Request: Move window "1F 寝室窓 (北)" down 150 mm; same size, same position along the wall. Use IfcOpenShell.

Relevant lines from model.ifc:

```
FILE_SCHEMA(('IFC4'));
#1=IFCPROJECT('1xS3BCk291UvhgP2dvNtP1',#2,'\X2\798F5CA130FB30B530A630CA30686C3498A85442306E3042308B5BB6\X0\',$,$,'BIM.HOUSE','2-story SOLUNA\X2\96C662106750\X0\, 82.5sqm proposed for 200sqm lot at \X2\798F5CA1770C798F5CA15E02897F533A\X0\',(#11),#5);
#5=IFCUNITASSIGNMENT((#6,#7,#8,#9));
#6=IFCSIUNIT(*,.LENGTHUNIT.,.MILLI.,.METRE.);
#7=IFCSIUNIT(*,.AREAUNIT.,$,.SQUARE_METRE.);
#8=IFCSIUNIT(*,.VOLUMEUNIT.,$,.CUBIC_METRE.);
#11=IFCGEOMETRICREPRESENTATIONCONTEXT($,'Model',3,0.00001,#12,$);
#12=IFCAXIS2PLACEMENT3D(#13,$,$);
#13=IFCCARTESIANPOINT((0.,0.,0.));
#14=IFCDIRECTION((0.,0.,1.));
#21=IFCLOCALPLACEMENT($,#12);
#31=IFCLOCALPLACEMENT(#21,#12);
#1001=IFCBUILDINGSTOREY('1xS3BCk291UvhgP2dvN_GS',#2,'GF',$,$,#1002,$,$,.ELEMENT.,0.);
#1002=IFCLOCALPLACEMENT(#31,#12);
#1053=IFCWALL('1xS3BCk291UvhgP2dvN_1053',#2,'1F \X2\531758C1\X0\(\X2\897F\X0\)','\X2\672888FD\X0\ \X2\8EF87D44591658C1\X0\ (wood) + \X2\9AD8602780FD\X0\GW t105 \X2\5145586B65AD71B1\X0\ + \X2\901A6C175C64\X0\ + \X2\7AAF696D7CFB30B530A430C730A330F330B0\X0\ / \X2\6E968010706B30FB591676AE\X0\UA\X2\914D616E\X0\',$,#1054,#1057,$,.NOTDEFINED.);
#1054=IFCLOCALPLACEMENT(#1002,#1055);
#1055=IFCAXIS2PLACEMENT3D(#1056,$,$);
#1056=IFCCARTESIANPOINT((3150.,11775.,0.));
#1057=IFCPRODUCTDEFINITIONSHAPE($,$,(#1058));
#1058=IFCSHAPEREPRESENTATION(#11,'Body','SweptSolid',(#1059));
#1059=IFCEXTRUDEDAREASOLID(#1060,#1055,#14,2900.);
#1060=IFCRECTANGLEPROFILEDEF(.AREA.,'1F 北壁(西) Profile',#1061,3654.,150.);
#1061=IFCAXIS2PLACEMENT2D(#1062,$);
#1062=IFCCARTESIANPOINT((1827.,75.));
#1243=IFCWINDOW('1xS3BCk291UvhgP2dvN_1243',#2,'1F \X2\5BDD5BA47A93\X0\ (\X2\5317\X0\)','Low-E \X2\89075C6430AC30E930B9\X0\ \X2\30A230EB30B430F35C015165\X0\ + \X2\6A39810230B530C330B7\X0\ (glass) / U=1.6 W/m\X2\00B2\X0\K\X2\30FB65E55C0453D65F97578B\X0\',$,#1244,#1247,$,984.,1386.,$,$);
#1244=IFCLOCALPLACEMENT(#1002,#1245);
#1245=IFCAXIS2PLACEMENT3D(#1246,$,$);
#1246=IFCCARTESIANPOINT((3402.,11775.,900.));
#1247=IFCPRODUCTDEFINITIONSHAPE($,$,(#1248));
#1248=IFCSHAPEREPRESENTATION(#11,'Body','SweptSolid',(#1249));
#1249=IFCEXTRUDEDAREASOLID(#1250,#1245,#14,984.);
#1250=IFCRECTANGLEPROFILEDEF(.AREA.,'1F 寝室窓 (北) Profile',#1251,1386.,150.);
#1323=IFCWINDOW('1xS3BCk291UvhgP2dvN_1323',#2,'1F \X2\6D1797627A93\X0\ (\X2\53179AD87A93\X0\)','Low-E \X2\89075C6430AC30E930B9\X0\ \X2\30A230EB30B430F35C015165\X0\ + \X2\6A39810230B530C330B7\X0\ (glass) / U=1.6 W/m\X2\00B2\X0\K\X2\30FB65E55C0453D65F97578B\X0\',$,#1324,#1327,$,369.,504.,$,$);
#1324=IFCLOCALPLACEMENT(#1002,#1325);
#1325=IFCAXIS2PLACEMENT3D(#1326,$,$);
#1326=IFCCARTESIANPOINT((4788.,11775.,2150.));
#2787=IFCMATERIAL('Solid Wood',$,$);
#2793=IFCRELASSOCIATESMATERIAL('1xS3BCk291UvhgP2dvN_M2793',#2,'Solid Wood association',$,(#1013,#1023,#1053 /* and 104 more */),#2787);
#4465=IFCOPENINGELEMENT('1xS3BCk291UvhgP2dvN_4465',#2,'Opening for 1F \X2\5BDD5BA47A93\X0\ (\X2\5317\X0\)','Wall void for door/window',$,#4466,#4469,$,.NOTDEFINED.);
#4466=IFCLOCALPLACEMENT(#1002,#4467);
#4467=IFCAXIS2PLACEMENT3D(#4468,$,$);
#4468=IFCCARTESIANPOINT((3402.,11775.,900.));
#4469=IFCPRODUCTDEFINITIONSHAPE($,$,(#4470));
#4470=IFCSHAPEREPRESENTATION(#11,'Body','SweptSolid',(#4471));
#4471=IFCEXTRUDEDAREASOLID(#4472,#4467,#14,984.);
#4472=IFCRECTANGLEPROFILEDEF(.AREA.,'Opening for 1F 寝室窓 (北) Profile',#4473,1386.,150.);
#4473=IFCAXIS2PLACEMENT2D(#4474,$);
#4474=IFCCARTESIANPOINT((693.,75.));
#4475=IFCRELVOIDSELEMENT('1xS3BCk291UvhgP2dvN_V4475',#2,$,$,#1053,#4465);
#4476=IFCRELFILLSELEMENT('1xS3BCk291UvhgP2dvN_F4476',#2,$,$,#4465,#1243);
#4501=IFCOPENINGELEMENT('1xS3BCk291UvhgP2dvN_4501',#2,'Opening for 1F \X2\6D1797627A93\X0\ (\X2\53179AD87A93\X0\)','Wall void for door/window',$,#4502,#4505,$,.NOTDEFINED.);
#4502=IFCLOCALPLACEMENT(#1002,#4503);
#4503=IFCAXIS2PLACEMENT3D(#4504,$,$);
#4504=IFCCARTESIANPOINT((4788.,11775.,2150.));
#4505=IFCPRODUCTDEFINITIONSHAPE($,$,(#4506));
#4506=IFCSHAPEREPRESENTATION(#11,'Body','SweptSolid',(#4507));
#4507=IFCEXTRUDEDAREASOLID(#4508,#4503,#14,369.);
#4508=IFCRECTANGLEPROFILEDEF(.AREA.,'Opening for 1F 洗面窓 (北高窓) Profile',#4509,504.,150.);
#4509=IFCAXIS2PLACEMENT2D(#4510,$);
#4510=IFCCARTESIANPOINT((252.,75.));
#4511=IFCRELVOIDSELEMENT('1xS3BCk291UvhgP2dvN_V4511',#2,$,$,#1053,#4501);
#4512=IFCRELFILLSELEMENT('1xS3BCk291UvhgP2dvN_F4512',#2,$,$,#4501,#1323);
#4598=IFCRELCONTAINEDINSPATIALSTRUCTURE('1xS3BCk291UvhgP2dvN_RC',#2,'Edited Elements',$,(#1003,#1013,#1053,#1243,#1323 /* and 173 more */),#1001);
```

```python
import numpy as np
import ifcopenshell
import ifcopenshell.api.geometry
import ifcopenshell.util.placement
import ifcopenshell.util.unit

model = ifcopenshell.open("model.ifc")
unit_scale = ifcopenshell.util.unit.calculate_unit_scale(model)

window = model.by_id(1243)
opening = window.FillsVoids[0].RelatingOpeningElement
dz = -0.15 / unit_scale

shift = np.array([0.0, 0.0, dz])
# The window is not placed relative to its opening, so move both.
for product in (opening, window):
    matrix = ifcopenshell.util.placement.get_local_placement(product.ObjectPlacement)
    matrix[:3, 3] += shift
    ifcopenshell.api.geometry.edit_object_placement(model, product=product, matrix=matrix, is_si=False)

print(f"moved by {dz * unit_scale:+.3f} m")

model.write("model_v2.ifc")
```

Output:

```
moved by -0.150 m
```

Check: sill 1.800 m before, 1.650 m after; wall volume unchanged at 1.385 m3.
